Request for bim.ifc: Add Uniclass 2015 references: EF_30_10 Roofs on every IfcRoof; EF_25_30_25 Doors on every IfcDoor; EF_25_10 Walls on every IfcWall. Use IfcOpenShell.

First a look at what the model holds.

```python
import ifcopenshell

model = ifcopenshell.open("bim.ifc")
print(model.schema)
print("classifications:", [c.Name for c in model.by_type("IfcClassification")])
for ifc_class in ("IfcDoor", "IfcRoof", "IfcStair", "IfcWall", "IfcWindow"):
    print(ifc_class, len(model.by_type(ifc_class)))
```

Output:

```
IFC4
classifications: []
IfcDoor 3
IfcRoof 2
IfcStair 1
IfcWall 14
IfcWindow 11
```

```python
import ifcopenshell
import ifcopenshell.api.classification

model = ifcopenshell.open("bim.ifc")

system = ifcopenshell.api.classification.add_classification(model, classification="Uniclass 2015")

codes = {
    "IfcRoof": ("EF_30_10", "Roofs"),
    "IfcDoor": ("EF_25_30_25", "Doors"),
    "IfcWall": ("EF_25_10", "Walls"),
}
for ifc_class, (code, name) in codes.items():
    products = model.by_type(ifc_class)
    ifcopenshell.api.classification.add_reference(
        model, products=products, classification=system, identification=code, name=name
    )
    print(code, len(products))

model.write("bim_v2.ifc")
```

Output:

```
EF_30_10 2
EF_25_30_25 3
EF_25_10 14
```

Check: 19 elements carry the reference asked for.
